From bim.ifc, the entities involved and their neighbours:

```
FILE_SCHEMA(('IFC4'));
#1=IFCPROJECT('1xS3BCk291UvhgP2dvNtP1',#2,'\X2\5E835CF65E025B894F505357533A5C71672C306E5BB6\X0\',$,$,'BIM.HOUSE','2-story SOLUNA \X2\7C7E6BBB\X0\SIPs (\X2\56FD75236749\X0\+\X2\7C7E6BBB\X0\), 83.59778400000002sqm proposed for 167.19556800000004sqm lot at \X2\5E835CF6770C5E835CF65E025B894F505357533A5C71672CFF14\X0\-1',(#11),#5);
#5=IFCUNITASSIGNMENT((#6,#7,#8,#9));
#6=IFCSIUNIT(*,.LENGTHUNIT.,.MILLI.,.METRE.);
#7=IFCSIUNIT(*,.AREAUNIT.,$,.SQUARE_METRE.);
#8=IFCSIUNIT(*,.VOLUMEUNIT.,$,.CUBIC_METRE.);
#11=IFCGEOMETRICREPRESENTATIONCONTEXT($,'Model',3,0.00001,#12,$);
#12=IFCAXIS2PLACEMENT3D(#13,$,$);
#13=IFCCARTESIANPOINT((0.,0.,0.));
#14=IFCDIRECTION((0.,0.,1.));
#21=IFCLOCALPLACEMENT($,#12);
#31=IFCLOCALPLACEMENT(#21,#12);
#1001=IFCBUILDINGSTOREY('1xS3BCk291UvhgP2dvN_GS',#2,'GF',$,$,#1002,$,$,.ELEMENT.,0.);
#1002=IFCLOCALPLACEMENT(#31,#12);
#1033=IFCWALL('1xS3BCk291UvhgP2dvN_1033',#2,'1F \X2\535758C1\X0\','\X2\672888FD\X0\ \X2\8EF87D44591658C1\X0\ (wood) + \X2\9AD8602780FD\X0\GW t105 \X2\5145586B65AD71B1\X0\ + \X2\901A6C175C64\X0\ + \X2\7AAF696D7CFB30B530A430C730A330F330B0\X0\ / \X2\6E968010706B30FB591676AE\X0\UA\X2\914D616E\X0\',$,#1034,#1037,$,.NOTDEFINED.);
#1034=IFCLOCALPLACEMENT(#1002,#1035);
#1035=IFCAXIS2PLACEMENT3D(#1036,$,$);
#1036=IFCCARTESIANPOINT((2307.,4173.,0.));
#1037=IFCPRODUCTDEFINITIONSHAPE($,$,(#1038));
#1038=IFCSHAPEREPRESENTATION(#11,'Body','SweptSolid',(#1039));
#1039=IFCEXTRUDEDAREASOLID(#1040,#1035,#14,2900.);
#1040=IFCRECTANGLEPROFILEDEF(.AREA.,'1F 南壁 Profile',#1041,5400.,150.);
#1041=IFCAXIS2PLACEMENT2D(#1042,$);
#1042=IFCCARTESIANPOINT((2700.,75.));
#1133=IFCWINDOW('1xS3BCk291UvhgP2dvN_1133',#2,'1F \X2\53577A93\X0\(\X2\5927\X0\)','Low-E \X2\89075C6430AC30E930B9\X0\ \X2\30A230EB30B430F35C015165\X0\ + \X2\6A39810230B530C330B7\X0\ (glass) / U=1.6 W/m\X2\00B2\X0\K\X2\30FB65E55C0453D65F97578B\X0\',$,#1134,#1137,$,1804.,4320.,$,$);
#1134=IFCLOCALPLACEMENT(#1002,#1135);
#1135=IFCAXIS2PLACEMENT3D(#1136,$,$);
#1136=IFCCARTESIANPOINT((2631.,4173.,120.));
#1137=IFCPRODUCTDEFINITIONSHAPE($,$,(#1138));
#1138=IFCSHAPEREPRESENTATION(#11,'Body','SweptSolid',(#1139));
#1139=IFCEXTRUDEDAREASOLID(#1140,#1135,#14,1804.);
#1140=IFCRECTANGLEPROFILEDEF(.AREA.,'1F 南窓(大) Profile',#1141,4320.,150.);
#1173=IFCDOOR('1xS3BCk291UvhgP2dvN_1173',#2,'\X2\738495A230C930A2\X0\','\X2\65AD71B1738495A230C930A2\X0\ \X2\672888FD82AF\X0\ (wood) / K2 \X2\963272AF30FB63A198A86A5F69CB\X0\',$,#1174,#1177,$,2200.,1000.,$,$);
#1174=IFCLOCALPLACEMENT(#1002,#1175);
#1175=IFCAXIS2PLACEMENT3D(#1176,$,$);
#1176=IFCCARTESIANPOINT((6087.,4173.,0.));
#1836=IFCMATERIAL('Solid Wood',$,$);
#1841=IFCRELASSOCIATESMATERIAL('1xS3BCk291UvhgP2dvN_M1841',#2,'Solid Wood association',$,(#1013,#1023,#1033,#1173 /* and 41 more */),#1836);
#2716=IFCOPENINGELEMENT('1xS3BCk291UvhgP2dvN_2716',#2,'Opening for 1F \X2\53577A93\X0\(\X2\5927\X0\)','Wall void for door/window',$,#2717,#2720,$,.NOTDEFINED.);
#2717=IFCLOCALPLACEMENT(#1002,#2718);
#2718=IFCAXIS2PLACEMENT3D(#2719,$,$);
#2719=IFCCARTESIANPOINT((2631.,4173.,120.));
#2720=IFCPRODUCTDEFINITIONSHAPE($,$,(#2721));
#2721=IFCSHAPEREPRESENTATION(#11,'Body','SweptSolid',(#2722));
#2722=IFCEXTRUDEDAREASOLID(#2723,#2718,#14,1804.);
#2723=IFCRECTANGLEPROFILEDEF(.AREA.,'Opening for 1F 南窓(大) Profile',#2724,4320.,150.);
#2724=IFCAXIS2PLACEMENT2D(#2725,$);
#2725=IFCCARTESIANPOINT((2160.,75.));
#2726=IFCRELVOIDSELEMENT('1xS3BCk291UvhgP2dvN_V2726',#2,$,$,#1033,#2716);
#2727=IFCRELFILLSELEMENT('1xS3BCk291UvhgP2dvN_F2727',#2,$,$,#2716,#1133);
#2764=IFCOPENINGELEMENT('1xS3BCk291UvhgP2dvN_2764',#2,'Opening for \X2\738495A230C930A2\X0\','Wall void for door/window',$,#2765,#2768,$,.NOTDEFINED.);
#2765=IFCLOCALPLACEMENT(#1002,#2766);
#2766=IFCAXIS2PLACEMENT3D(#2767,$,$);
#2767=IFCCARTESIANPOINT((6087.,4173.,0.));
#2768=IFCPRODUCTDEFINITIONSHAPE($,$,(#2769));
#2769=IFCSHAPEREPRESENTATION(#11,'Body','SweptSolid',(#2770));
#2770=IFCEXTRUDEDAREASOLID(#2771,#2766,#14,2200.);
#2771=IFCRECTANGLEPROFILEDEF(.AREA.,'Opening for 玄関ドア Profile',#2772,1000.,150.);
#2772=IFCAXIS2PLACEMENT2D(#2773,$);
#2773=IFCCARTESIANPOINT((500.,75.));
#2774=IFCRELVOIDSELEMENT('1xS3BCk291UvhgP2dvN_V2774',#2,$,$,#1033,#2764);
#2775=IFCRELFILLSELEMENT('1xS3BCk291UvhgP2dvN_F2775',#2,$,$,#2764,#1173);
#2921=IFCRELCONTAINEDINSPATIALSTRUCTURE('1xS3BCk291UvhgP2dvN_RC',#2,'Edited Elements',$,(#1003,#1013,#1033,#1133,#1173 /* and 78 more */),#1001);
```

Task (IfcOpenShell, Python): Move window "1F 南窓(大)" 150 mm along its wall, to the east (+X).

```python
import ifcopenshell
import ifcopenshell.api.geometry
import ifcopenshell.util.placement

model = ifcopenshell.open("bim.ifc")

window = model.by_id(1133)
opening = window.FillsVoids[0].RelatingOpeningElement
wall = opening.VoidsElements[0].RelatingBuildingElement

wall_matrix = ifcopenshell.util.placement.get_local_placement(wall.ObjectPlacement)
shift = wall_matrix[:3, 0] * 150.0
before = ifcopenshell.util.placement.get_local_placement(window.ObjectPlacement)[:3, 3].copy()

# The window is not placed relative to its opening, so move both.
for product in (opening, window):
    matrix = ifcopenshell.util.placement.get_local_placement(product.ObjectPlacement)
    matrix[:3, 3] += shift
    ifcopenshell.api.geometry.edit_object_placement(model, product=product, matrix=matrix, is_si=False)

after = ifcopenshell.util.placement.get_local_placement(window.ObjectPlacement)[:3, 3]
print("window moved by", (after - before).round(3) + 0.0)

model.write("bim_updated.ifc")
```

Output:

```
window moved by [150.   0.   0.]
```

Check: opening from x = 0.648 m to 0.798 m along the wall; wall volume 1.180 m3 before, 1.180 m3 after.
